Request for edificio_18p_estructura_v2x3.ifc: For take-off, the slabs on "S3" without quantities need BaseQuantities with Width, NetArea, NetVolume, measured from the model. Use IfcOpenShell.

First a look at what the model holds.

```python
import ifcopenshell
import ifcopenshell.util.element
import ifcopenshell.util.unit

model = ifcopenshell.open("edificio_18p_estructura_v2x3.ifc")
print(model.schema)
for unit_type in ("LENGTHUNIT", "AREAUNIT", "VOLUMEUNIT"):
    print(unit_type, ifcopenshell.util.unit.calculate_unit_scale(model, unit_type))
storey = next(s for s in model.by_type("IfcBuildingStorey") if s.Name == "S3")
slabs = [e for e in ifcopenshell.util.element.get_decomposition(storey) if e.is_a("IfcSlab")]
for e in sorted(slabs, key=lambda e: e.id()):
    print(e.id(), e.is_a(), e.Name, list(ifcopenshell.util.element.get_psets(e, qtos_only=True)), sep=" | ")
```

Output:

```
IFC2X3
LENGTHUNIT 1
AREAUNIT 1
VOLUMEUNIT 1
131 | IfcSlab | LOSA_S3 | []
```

```python
import ifcopenshell
import ifcopenshell.api.pset
import ifcopenshell.geom
import ifcopenshell.util.element
import ifcopenshell.util.shape
import ifcopenshell.util.unit

model = ifcopenshell.open("edificio_18p_estructura_v2x3.ifc")
unit_scale = ifcopenshell.util.unit.calculate_unit_scale(model)
area_scale = ifcopenshell.util.unit.calculate_unit_scale(model, "AREAUNIT")
volume_scale = ifcopenshell.util.unit.calculate_unit_scale(model, "VOLUMEUNIT")
settings = ifcopenshell.geom.settings()

storey = next(s for s in model.by_type("IfcBuildingStorey") if s.Name == "S3")
slabs = [e for e in ifcopenshell.util.element.get_decomposition(storey) if e.is_a("IfcSlab")]

for e in sorted(slabs, key=lambda e: e.id()):
    if ifcopenshell.util.element.get_psets(e, qtos_only=True, should_inherit=False):
        continue
    # Geometry comes back in metres, in the element's own axes.
    shape = ifcopenshell.geom.create_shape(settings, e)
    values = {
        "Width": ifcopenshell.util.shape.get_z(shape.geometry) / unit_scale,
        "NetArea": ifcopenshell.util.shape.get_footprint_area(shape.geometry) / area_scale,
        "NetVolume": ifcopenshell.util.shape.get_volume(shape.geometry) / volume_scale,
    }
    qto = ifcopenshell.api.pset.add_qto(model, product=e, name="BaseQuantities")
    ifcopenshell.api.pset.edit_qto(model, qto=qto, properties=values)
    print(e.id(), {k: round(v, 3) for k, v in values.items()})

model.write("edificio_18p_estructura_v2x3_updated.ifc")
```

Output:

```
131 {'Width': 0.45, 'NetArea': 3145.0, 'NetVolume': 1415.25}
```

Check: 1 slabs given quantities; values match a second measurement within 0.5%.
